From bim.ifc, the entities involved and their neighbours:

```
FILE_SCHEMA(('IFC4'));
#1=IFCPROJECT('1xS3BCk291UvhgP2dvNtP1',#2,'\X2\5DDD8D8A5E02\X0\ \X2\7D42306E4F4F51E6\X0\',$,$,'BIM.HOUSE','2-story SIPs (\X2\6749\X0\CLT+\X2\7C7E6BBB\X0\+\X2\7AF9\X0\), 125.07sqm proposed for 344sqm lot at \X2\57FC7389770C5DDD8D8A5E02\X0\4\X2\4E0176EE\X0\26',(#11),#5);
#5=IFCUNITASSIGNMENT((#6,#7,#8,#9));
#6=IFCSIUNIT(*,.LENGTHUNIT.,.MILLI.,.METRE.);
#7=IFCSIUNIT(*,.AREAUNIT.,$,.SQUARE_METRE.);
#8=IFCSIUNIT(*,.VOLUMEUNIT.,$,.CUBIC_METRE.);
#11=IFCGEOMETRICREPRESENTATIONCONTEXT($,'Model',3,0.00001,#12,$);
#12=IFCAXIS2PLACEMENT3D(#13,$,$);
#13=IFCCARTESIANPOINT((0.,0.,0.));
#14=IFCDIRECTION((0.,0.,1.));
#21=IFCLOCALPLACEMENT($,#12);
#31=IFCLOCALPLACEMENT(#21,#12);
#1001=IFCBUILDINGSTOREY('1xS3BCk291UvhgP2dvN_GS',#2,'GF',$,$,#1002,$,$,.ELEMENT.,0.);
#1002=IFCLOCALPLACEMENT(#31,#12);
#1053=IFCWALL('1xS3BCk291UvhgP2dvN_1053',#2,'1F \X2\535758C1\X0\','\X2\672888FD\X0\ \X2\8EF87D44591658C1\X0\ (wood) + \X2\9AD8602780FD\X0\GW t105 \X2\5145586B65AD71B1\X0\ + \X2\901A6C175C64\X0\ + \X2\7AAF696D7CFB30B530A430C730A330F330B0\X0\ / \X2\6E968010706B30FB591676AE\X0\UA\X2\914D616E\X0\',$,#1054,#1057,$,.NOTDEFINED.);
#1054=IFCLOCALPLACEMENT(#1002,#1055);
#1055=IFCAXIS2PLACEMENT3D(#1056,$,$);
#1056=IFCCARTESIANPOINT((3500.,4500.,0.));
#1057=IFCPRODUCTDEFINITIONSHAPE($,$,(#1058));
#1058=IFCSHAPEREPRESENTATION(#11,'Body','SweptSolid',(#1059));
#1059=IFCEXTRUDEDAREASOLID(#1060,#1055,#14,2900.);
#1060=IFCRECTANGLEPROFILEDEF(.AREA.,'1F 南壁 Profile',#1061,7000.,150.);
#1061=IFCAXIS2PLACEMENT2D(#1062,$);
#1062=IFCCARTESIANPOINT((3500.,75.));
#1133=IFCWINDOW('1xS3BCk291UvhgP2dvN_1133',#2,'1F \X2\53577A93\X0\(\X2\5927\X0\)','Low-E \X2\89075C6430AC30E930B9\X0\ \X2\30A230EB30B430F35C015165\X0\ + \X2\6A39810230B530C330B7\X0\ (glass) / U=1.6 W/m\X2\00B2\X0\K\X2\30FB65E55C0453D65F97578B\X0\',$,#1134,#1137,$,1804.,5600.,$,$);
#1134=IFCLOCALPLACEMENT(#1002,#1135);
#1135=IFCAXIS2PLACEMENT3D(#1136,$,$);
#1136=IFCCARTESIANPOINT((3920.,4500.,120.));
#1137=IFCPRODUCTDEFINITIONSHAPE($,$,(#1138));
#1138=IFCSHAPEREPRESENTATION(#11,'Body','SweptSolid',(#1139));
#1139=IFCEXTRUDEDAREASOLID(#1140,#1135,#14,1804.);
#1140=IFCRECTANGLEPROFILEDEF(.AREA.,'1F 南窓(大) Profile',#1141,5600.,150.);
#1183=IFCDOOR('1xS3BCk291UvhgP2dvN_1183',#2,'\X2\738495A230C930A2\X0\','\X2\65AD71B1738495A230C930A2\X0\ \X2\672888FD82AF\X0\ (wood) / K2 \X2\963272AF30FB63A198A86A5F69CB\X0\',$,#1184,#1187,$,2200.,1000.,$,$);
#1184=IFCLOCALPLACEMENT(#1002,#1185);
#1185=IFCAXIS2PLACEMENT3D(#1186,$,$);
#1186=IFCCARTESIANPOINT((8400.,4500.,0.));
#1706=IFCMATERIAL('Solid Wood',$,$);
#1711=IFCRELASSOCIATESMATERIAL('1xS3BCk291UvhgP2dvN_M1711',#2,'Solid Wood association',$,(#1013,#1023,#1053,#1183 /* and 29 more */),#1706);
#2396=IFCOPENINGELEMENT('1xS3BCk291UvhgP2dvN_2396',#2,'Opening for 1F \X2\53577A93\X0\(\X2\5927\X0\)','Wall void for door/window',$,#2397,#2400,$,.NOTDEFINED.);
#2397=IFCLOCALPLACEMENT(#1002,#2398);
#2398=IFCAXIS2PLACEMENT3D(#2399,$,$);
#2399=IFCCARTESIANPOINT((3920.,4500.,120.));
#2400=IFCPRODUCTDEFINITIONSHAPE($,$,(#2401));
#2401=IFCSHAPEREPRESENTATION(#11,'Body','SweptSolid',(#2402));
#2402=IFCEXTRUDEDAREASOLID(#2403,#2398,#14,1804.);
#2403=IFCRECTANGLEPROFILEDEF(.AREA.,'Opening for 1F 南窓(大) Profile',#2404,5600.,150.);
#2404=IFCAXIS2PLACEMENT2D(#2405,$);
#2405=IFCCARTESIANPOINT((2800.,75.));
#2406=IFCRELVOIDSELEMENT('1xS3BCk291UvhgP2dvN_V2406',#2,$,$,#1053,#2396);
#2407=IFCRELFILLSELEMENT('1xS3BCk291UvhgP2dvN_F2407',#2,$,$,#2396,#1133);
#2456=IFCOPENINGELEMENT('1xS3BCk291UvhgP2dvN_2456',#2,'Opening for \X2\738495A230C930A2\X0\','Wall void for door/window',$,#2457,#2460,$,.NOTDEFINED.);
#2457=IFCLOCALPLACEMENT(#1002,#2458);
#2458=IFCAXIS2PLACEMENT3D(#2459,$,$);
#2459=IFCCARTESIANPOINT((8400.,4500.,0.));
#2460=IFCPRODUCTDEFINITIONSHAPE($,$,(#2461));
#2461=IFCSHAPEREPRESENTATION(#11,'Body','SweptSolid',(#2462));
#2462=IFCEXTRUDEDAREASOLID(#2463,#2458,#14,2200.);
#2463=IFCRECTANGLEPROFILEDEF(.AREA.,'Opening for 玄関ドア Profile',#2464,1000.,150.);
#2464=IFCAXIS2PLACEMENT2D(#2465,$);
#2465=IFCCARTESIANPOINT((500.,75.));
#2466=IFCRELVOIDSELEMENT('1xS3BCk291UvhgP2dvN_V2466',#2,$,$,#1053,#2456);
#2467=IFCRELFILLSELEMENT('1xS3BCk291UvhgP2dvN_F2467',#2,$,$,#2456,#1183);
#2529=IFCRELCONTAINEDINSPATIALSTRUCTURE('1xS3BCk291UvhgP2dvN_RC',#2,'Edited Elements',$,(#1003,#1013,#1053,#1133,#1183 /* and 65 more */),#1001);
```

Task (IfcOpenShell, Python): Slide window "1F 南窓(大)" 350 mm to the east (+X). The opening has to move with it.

```python
import ifcopenshell
import ifcopenshell.api.geometry
import ifcopenshell.util.placement

model = ifcopenshell.open("bim.ifc")

window = model.by_guid("1xS3BCk291UvhgP2dvN_1133")
opening = window.FillsVoids[0].RelatingOpeningElement
wall = opening.VoidsElements[0].RelatingBuildingElement

wall_matrix = ifcopenshell.util.placement.get_local_placement(wall.ObjectPlacement)
shift = wall_matrix[:3, 0] * 350.0
before = ifcopenshell.util.placement.get_local_placement(window.ObjectPlacement)[:3, 3].copy()

# The window is not placed relative to its opening, so move both.
for product in (opening, window):
    matrix = ifcopenshell.util.placement.get_local_placement(product.ObjectPlacement)
    matrix[:3, 3] += shift
    ifcopenshell.api.geometry.edit_object_placement(model, product=product, matrix=matrix, is_si=False)

after = ifcopenshell.util.placement.get_local_placement(window.ObjectPlacement)[:3, 3]
print("window moved by", (after - before).round(3) + 0.0)

model.write("bim_updated.ifc")
```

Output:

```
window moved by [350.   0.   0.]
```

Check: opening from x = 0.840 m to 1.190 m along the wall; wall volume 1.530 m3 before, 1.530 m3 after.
